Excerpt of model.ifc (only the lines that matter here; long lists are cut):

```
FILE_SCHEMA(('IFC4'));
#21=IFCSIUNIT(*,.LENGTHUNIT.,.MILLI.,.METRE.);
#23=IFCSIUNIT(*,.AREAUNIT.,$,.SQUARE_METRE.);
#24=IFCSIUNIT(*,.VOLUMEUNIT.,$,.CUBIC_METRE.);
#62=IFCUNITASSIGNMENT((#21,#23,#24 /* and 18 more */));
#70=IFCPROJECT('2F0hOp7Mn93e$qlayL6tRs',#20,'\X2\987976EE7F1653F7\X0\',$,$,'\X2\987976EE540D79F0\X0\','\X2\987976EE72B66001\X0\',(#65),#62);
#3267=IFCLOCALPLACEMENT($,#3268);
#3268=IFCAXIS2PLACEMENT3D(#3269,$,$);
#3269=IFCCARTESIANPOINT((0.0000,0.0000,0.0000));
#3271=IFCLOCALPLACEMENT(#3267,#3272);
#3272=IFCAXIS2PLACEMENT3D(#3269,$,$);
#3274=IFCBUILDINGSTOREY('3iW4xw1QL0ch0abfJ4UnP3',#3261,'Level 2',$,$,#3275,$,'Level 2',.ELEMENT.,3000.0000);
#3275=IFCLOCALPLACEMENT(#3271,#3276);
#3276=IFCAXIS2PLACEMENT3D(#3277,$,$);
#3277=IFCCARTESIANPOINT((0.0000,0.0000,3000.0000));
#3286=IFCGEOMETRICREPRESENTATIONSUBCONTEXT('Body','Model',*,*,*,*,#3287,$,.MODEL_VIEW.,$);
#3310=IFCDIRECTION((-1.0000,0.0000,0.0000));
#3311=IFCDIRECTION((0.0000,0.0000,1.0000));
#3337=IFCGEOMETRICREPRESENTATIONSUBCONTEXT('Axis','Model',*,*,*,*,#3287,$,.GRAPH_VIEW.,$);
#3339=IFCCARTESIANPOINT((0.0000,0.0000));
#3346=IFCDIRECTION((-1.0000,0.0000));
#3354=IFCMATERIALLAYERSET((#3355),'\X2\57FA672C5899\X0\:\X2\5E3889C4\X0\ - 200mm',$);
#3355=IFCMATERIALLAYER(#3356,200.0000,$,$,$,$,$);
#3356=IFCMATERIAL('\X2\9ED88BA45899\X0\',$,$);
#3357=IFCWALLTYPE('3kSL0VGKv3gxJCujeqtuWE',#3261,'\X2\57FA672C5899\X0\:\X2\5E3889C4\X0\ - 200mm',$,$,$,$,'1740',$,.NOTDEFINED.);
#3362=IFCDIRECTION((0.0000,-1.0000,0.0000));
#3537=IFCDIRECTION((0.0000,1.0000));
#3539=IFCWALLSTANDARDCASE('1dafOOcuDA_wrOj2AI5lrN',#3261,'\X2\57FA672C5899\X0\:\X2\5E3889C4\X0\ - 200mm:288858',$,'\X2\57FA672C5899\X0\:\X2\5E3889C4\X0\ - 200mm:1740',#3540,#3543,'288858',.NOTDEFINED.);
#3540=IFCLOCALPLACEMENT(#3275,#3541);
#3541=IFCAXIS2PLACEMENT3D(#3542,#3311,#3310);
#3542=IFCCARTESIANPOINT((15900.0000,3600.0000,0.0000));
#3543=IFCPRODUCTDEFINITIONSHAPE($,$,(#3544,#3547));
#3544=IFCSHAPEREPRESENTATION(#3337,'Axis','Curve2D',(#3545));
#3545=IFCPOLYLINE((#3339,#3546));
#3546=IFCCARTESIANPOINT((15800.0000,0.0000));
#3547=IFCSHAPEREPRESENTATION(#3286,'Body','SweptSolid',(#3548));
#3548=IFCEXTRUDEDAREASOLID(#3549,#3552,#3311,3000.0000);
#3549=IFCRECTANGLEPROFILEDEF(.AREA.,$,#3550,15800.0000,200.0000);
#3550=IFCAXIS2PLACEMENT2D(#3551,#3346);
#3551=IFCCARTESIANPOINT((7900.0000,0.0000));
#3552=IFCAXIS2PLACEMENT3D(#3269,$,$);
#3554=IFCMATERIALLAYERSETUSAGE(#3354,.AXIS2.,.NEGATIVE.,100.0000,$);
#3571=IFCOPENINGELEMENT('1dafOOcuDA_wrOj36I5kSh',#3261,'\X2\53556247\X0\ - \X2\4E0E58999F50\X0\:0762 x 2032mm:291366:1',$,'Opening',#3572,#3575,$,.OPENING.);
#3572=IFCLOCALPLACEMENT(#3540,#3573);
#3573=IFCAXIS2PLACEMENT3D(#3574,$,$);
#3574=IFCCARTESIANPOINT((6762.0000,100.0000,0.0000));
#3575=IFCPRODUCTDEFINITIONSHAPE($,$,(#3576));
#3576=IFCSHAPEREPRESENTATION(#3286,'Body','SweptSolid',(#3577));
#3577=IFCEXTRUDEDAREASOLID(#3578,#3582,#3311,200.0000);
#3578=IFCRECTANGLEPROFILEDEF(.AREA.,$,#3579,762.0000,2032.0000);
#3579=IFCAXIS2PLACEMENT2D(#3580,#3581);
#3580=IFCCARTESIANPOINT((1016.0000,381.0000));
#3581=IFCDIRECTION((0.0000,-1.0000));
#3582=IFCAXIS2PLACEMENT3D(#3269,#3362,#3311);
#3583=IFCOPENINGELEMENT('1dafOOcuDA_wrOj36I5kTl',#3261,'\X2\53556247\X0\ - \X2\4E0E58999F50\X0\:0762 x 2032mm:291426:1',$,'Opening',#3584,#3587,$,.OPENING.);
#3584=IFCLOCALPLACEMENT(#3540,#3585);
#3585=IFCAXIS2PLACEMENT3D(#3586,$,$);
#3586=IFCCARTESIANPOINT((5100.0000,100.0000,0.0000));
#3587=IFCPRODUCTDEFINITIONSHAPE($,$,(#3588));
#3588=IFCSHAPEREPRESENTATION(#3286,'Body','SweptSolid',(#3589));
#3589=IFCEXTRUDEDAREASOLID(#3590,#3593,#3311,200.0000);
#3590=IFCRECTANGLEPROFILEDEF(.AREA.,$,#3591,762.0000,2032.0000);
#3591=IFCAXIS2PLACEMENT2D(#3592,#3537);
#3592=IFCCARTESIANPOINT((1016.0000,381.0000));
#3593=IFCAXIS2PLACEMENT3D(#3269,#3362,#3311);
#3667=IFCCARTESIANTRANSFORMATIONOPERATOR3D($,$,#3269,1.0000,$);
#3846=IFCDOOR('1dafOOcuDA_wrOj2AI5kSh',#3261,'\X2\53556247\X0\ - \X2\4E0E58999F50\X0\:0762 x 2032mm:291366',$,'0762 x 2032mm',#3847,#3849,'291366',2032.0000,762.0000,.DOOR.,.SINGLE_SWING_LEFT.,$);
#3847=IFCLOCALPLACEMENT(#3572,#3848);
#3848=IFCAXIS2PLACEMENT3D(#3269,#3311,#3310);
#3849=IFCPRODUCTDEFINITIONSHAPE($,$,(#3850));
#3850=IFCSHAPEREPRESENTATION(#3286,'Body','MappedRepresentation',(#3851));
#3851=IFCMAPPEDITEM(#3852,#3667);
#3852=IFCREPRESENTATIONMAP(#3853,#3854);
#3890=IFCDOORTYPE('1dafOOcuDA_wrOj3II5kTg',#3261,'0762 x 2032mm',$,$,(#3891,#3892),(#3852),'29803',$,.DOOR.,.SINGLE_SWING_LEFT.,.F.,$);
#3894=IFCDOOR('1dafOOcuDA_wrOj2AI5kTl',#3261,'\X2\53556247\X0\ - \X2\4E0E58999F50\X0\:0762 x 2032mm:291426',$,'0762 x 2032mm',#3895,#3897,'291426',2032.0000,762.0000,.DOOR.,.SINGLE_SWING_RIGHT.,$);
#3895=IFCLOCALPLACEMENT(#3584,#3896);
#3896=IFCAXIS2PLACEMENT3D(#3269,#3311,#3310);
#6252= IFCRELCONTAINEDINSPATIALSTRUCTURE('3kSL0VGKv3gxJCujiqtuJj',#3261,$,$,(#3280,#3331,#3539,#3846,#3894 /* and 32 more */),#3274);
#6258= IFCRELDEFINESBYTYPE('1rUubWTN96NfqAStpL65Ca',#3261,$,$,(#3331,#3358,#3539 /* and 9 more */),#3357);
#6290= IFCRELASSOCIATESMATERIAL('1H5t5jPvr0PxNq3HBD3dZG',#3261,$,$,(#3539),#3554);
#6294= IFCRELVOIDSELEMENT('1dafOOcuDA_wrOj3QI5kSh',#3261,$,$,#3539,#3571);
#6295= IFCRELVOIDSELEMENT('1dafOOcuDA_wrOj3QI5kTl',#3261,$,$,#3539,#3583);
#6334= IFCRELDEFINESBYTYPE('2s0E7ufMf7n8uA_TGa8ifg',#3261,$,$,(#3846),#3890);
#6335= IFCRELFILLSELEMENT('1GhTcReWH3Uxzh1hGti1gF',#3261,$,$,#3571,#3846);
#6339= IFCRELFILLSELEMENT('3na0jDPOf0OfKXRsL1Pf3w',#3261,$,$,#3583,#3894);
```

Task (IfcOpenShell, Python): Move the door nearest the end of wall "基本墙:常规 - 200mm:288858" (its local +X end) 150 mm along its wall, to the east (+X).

```python
import ifcopenshell
import ifcopenshell.api.geometry
import ifcopenshell.util.placement
import ifcopenshell.util.unit

model = ifcopenshell.open("model.ifc")
unit_scale = ifcopenshell.util.unit.calculate_unit_scale(model)

door = model.by_guid("1dafOOcuDA_wrOj2AI5kSh")
opening = door.FillsVoids[0].RelatingOpeningElement
wall = opening.VoidsElements[0].RelatingBuildingElement

wall_matrix = ifcopenshell.util.placement.get_local_placement(wall.ObjectPlacement)
shift = wall_matrix[:3, 0] * -0.15 / unit_scale
before = ifcopenshell.util.placement.get_local_placement(door.ObjectPlacement)[:3, 3].copy()

# The door is placed relative to its opening, so it follows when the opening moves.
matrix = ifcopenshell.util.placement.get_local_placement(opening.ObjectPlacement)
matrix[:3, 3] += shift
ifcopenshell.api.geometry.edit_object_placement(
    model, product=opening, matrix=matrix, is_si=False, should_transform_children=True
)

after = ifcopenshell.util.placement.get_local_placement(door.ObjectPlacement)[:3, 3]
print("door moved by", (after - before).round(3) + 0.0)

model.write("model_updated.ifc")
```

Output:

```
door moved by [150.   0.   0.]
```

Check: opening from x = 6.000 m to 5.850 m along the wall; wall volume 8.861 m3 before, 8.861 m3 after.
